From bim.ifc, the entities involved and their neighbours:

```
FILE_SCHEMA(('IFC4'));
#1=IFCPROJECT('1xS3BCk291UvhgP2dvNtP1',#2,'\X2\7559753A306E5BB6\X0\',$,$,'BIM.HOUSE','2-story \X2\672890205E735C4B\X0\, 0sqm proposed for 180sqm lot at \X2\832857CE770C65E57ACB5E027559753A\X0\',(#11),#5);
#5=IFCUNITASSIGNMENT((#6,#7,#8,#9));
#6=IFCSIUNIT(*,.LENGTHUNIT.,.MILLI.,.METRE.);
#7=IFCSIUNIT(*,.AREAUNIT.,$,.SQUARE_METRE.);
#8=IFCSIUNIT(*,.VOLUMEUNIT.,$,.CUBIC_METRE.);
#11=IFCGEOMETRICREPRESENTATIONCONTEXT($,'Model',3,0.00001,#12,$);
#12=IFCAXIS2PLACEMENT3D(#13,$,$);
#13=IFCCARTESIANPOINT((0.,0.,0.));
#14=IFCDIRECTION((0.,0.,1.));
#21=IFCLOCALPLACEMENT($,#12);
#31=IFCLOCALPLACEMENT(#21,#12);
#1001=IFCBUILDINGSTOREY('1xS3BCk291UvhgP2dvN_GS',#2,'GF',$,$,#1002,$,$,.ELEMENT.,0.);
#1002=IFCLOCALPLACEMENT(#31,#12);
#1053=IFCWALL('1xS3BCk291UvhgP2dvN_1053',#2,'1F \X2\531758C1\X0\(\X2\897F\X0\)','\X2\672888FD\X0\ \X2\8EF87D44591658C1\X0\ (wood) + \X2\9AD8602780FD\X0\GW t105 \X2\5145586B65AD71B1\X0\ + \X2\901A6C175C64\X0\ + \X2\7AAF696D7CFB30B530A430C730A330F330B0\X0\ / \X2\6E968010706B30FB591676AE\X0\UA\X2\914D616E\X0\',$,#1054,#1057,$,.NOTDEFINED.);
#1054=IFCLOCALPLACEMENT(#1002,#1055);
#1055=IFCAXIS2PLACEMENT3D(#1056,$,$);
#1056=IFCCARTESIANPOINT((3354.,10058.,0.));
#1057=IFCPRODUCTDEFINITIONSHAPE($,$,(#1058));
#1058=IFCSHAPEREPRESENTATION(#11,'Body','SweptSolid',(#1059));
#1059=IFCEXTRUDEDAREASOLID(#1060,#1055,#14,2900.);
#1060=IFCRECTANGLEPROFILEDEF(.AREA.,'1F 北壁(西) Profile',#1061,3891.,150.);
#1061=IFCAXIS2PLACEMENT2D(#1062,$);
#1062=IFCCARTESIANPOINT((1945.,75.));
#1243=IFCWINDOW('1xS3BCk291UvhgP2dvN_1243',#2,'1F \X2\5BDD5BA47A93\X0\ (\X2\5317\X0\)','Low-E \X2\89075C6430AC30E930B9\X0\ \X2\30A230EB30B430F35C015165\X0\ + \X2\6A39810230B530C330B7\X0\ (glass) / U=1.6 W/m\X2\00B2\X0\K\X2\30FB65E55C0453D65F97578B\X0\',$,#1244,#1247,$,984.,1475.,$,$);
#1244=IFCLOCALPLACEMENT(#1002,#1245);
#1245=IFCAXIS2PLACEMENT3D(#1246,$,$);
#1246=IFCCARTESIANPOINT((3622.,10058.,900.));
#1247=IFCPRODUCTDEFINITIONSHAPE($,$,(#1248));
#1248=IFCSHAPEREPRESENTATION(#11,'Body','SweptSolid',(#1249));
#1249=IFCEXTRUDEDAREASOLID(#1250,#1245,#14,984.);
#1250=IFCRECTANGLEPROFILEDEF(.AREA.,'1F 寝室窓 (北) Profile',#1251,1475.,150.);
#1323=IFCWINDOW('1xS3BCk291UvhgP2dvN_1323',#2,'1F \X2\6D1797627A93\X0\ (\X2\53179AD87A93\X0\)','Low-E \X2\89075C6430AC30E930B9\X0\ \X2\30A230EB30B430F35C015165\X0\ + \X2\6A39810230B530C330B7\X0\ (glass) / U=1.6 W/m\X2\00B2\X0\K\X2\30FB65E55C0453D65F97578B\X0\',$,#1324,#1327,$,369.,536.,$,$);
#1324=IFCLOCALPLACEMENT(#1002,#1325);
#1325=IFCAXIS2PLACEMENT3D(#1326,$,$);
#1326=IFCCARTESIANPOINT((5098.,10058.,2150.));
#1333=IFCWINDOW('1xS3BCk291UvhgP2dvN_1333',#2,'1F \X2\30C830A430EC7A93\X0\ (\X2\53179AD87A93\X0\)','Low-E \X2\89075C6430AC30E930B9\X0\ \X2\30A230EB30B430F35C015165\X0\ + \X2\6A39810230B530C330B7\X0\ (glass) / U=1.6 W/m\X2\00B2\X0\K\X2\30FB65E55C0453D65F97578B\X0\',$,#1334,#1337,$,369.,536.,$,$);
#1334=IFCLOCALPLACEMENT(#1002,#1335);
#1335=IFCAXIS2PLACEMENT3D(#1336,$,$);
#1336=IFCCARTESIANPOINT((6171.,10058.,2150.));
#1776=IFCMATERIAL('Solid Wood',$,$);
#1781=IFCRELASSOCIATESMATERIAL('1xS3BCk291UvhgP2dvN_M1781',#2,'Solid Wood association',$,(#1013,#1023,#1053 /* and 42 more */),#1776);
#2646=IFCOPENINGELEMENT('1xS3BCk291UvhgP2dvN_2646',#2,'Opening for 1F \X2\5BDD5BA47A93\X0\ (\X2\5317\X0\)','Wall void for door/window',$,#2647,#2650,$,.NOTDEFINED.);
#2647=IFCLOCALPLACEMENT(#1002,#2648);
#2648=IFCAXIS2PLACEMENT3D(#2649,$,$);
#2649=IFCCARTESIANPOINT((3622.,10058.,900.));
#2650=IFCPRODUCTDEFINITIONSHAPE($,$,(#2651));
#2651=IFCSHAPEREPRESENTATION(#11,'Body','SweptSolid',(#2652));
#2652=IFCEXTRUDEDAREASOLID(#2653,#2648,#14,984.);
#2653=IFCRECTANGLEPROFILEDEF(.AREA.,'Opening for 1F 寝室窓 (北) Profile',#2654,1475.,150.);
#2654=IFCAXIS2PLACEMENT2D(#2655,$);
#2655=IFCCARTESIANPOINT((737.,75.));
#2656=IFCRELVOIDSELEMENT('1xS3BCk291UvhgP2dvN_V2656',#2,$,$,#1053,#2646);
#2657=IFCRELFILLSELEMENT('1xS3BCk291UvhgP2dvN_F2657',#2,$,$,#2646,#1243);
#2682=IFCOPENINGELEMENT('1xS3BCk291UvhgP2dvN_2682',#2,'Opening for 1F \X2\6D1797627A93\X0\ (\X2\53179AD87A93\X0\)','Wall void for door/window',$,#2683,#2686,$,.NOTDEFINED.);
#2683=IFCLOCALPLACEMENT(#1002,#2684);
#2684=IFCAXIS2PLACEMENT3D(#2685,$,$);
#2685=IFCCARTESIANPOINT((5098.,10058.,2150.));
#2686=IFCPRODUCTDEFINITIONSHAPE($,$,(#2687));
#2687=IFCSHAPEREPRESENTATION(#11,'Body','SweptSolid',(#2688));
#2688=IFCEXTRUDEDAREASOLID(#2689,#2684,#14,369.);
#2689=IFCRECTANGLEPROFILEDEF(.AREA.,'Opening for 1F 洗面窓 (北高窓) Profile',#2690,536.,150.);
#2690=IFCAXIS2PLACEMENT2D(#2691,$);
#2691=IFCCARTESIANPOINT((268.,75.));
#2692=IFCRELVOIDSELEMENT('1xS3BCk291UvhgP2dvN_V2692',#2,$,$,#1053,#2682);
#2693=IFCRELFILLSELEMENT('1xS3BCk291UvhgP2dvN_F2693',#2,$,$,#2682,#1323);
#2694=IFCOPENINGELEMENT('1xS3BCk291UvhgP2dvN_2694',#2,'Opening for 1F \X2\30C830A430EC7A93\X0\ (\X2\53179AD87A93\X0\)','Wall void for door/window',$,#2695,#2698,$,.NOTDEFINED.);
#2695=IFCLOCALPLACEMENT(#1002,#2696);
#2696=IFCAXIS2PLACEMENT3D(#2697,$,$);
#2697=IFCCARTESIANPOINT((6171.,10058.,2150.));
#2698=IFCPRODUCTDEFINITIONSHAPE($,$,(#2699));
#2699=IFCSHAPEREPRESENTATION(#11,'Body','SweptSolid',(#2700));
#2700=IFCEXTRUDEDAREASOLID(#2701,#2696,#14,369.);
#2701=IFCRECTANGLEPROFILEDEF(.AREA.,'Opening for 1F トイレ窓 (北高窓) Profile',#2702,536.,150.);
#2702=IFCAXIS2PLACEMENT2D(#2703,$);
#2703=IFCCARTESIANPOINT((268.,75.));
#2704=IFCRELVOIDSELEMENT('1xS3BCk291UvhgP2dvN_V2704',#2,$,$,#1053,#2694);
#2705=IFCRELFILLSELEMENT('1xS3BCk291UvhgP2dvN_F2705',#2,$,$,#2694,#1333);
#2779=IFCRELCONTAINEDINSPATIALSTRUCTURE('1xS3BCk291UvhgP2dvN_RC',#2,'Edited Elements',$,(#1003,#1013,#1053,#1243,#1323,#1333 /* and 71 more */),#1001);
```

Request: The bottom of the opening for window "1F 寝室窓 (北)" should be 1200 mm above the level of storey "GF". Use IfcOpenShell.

```python
import numpy as np
import ifcopenshell
import ifcopenshell.api.geometry
import ifcopenshell.geom
import ifcopenshell.util.element
import ifcopenshell.util.placement
import ifcopenshell.util.shape
import ifcopenshell.util.unit

model = ifcopenshell.open("bim.ifc")
unit_scale = ifcopenshell.util.unit.calculate_unit_scale(model)

window = model.by_guid("1xS3BCk291UvhgP2dvN_1243")
opening = window.FillsVoids[0].RelatingOpeningElement
storey = ifcopenshell.util.element.get_container(window, ifc_class="IfcBuildingStorey")
level = ifcopenshell.util.placement.get_local_placement(storey.ObjectPlacement)[2, 3]

# The opening's origin need not be at the sill, so measure its lowest point.
shape = ifcopenshell.geom.create_shape(ifcopenshell.geom.settings(), opening)
bottom = ifcopenshell.util.shape.get_shape_bottom_elevation(shape, shape.geometry) / unit_scale
dz = level + 1.2 / unit_scale - bottom

shift = np.array([0.0, 0.0, dz])
# The window is not placed relative to its opening, so move both.
for product in (opening, window):
    matrix = ifcopenshell.util.placement.get_local_placement(product.ObjectPlacement)
    matrix[:3, 3] += shift
    ifcopenshell.api.geometry.edit_object_placement(model, product=product, matrix=matrix, is_si=False)

print(f"moved by {dz * unit_scale:+.3f} m")

model.write("bim-out.ifc")
```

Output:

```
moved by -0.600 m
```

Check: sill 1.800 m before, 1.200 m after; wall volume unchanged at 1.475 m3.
